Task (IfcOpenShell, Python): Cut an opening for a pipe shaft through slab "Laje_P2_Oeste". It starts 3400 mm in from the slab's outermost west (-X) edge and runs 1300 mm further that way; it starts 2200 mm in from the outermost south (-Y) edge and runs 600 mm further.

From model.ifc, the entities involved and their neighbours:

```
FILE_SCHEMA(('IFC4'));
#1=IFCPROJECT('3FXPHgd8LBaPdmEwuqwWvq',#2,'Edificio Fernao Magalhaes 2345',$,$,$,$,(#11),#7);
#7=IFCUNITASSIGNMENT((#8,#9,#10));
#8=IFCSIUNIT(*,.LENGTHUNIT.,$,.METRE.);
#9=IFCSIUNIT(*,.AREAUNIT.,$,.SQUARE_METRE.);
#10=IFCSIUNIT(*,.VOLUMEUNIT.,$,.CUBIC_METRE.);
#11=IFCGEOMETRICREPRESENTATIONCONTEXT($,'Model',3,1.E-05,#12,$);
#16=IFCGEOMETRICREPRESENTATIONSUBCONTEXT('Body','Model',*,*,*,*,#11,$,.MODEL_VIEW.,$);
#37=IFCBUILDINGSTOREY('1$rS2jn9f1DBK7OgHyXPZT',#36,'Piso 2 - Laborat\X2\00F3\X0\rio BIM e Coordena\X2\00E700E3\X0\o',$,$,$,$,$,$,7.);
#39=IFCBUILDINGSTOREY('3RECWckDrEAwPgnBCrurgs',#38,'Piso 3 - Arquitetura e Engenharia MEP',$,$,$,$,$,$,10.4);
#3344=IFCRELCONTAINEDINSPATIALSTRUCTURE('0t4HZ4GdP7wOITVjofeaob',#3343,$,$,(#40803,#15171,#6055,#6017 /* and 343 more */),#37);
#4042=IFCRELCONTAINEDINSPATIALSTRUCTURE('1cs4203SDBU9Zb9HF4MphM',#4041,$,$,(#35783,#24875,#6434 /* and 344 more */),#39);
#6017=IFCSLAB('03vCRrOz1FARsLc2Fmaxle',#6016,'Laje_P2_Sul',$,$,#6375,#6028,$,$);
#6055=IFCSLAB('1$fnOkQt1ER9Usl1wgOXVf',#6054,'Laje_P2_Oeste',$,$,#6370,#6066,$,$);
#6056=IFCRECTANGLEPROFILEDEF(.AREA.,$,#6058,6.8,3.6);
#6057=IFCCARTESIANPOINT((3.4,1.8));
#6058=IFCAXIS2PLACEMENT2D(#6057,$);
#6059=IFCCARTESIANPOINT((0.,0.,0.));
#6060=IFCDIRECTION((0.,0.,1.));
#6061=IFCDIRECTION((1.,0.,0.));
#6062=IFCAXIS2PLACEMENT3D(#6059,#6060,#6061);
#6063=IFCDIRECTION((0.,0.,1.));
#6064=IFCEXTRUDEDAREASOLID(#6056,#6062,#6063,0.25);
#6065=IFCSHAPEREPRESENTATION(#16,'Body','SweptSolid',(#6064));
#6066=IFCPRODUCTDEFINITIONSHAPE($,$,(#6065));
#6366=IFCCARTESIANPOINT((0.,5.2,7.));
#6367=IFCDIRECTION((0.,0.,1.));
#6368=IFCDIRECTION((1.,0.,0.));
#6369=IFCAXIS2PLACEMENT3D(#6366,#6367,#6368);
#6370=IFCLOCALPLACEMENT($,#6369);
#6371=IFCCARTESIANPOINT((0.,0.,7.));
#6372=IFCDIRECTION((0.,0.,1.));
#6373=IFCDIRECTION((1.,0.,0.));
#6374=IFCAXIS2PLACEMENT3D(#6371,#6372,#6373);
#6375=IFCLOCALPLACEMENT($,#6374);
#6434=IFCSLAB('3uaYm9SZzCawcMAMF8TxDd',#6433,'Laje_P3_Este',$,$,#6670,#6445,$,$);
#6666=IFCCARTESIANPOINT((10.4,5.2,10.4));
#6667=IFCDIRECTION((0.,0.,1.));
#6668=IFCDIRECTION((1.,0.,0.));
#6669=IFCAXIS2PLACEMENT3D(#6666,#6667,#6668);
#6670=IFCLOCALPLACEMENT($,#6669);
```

```python
import numpy as np
import ifcopenshell
import ifcopenshell.api.feature
import ifcopenshell.api.geometry
import ifcopenshell.api.root
import ifcopenshell.geom
import ifcopenshell.util.placement
import ifcopenshell.util.representation
import ifcopenshell.util.shape
import ifcopenshell.util.unit

model = ifcopenshell.open("model.ifc")
unit_scale = ifcopenshell.util.unit.calculate_unit_scale(model)
settings = ifcopenshell.geom.settings()


def volume(element):
    """Net volume in cubic metres, openings subtracted."""
    shape = ifcopenshell.geom.create_shape(settings, element)
    return ifcopenshell.util.shape.get_volume(shape.geometry)


slab = model.by_id(6055)
before = volume(slab)

# Extent in the slab's own axes, in metres. The edges named are its -X and -Y sides.
slab_shape = ifcopenshell.geom.create_shape(settings, slab)
vertices = ifcopenshell.util.shape.get_vertices(slab_shape.geometry)
x_min, y_min, bottom = vertices.min(axis=0)
top = vertices[:, 2].max()

opening = ifcopenshell.api.root.create_entity(model, ifc_class="IfcOpeningElement", name="Pipe shaft opening", predefined_type="OPENING")
context = ifcopenshell.util.representation.get_context(model, "Model", "Body", "MODEL_VIEW")
width, depth = 1.3, 0.6
outline = [(0.0, 0.0), (width, 0.0), (width, depth), (0.0, depth), (0.0, 0.0)]
# Overshoot both faces by 50 mm so the cut is clean.
shape = ifcopenshell.api.geometry.add_slab_representation(
    model, context=context, depth=top - bottom + 0.1, polyline=outline
)
ifcopenshell.api.geometry.assign_representation(model, product=opening, representation=shape)

matrix = ifcopenshell.util.placement.get_local_placement(slab.ObjectPlacement)
matrix[:, 3] = matrix @ np.append(np.array([x_min + 3.4, y_min + 2.2, bottom - 0.05]) / unit_scale, 1.0)
ifcopenshell.api.geometry.edit_object_placement(model, product=opening, matrix=matrix, is_si=False)
ifcopenshell.api.feature.add_feature(model, feature=opening, element=slab)

after = volume(slab)

print(f"slab volume {before:.3f} -> {after:.3f} m3")

model.write("model_v2.ifc")
```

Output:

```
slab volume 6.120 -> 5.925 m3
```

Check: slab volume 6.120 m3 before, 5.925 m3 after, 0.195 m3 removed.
